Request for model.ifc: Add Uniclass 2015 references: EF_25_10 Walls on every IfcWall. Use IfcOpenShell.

First a look at what the model holds.

```python
import ifcopenshell

model = ifcopenshell.open("model.ifc")
print(model.schema)
print("classifications:", [c.Name for c in model.by_type("IfcClassification")])
for ifc_class in ("IfcDoor", "IfcRoof", "IfcStair", "IfcWall", "IfcWindow"):
    print(ifc_class, len(model.by_type(ifc_class)))
```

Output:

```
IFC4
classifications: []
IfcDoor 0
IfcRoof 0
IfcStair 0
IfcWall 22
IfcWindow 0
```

```python
import ifcopenshell
import ifcopenshell.api.classification

model = ifcopenshell.open("model.ifc")

system = ifcopenshell.api.classification.add_classification(model, classification="Uniclass 2015")

codes = {
    "IfcWall": ("EF_25_10", "Walls"),
}
for ifc_class, (code, name) in codes.items():
    products = model.by_type(ifc_class)
    ifcopenshell.api.classification.add_reference(
        model, products=products, classification=system, identification=code, name=name
    )
    print(code, len(products))

model.write("model_updated.ifc")
```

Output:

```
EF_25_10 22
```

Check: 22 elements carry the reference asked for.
